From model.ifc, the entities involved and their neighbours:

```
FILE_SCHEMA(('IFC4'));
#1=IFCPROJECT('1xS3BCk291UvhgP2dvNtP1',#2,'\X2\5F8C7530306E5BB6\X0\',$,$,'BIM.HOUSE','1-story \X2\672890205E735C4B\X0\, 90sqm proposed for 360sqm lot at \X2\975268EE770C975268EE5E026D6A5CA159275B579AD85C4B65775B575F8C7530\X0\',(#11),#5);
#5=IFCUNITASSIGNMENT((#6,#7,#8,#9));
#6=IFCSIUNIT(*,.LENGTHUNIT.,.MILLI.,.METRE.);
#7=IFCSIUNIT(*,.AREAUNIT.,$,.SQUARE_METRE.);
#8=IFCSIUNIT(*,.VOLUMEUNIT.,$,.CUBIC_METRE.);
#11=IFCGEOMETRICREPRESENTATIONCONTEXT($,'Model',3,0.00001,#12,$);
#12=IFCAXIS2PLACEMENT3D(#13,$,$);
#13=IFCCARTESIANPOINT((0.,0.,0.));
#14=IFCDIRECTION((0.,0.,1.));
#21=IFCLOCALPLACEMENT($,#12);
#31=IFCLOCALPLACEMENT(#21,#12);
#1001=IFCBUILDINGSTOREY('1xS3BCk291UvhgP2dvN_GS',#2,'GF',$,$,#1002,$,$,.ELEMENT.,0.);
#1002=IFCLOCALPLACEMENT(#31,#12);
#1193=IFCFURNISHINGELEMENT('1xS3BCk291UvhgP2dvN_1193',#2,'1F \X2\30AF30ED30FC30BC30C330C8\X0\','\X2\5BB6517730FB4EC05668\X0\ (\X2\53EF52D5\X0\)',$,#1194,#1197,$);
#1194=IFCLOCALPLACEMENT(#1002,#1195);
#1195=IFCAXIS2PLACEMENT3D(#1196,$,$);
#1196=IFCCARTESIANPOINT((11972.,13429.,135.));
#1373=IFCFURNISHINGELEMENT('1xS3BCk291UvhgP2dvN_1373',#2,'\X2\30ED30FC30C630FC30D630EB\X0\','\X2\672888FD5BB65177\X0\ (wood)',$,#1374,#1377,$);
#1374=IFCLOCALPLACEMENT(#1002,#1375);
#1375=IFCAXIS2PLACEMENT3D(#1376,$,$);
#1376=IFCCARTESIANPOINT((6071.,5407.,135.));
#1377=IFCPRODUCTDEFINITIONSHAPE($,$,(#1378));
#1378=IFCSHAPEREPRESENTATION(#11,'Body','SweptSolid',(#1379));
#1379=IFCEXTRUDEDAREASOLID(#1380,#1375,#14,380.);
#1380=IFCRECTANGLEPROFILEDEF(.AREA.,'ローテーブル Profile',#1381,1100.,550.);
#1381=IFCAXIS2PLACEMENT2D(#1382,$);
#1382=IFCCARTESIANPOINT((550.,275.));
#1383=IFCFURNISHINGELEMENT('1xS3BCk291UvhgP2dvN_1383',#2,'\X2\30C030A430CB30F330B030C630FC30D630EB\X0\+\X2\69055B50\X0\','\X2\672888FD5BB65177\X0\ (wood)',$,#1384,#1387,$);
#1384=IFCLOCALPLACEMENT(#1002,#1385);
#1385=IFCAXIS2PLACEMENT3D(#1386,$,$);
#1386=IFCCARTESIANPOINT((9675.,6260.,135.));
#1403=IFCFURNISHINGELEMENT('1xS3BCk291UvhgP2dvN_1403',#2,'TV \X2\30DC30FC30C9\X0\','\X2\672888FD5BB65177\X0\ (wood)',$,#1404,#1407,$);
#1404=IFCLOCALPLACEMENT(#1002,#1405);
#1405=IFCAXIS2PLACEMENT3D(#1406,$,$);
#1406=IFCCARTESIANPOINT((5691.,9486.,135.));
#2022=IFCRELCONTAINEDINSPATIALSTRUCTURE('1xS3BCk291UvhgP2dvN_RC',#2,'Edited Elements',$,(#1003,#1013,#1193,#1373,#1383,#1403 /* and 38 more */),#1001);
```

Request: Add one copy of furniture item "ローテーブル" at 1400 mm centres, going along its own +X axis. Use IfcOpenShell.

```python
import ifcopenshell
import ifcopenshell.api.geometry
import ifcopenshell.api.root
import ifcopenshell.util.element
import ifcopenshell.util.placement
import ifcopenshell.util.unit

model = ifcopenshell.open("model.ifc")
unit_scale = ifcopenshell.util.unit.calculate_unit_scale(model)


def reuse_history(source, copy):
    """copy_class also copies each property set's owner history, people and application; keep the originals."""
    for rel in copy.IsDefinedBy:
        if rel.is_a("IfcRelDefinesByProperties") and (history := rel.RelatingPropertyDefinition.OwnerHistory):
            rel.RelatingPropertyDefinition.OwnerHistory = source.OwnerHistory
            ifcopenshell.util.element.remove_deep2(model, history)


source = model.by_guid("1xS3BCk291UvhgP2dvN_1373")
base = ifcopenshell.util.placement.get_local_placement(source.ObjectPlacement)
step = base[:3, 0] * 1.4 / unit_scale

for i in range(1, 2):
    copy = ifcopenshell.api.root.copy_class(model, product=source)
    copy.Representation = ifcopenshell.util.element.copy_deep(
        model, source.Representation, exclude=["IfcGeometricRepresentationContext", "IfcRepresentationMap"]
    )
    reuse_history(source, copy)
    matrix = base.copy()
    matrix[:3, 3] += i * step
    print("added at", matrix[:3, 3].round(3) + 0.0)
    ifcopenshell.api.geometry.edit_object_placement(model, product=copy, matrix=matrix, is_si=False)

model.write("model_v2.ifc")
```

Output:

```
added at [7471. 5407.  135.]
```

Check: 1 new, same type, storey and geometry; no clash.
